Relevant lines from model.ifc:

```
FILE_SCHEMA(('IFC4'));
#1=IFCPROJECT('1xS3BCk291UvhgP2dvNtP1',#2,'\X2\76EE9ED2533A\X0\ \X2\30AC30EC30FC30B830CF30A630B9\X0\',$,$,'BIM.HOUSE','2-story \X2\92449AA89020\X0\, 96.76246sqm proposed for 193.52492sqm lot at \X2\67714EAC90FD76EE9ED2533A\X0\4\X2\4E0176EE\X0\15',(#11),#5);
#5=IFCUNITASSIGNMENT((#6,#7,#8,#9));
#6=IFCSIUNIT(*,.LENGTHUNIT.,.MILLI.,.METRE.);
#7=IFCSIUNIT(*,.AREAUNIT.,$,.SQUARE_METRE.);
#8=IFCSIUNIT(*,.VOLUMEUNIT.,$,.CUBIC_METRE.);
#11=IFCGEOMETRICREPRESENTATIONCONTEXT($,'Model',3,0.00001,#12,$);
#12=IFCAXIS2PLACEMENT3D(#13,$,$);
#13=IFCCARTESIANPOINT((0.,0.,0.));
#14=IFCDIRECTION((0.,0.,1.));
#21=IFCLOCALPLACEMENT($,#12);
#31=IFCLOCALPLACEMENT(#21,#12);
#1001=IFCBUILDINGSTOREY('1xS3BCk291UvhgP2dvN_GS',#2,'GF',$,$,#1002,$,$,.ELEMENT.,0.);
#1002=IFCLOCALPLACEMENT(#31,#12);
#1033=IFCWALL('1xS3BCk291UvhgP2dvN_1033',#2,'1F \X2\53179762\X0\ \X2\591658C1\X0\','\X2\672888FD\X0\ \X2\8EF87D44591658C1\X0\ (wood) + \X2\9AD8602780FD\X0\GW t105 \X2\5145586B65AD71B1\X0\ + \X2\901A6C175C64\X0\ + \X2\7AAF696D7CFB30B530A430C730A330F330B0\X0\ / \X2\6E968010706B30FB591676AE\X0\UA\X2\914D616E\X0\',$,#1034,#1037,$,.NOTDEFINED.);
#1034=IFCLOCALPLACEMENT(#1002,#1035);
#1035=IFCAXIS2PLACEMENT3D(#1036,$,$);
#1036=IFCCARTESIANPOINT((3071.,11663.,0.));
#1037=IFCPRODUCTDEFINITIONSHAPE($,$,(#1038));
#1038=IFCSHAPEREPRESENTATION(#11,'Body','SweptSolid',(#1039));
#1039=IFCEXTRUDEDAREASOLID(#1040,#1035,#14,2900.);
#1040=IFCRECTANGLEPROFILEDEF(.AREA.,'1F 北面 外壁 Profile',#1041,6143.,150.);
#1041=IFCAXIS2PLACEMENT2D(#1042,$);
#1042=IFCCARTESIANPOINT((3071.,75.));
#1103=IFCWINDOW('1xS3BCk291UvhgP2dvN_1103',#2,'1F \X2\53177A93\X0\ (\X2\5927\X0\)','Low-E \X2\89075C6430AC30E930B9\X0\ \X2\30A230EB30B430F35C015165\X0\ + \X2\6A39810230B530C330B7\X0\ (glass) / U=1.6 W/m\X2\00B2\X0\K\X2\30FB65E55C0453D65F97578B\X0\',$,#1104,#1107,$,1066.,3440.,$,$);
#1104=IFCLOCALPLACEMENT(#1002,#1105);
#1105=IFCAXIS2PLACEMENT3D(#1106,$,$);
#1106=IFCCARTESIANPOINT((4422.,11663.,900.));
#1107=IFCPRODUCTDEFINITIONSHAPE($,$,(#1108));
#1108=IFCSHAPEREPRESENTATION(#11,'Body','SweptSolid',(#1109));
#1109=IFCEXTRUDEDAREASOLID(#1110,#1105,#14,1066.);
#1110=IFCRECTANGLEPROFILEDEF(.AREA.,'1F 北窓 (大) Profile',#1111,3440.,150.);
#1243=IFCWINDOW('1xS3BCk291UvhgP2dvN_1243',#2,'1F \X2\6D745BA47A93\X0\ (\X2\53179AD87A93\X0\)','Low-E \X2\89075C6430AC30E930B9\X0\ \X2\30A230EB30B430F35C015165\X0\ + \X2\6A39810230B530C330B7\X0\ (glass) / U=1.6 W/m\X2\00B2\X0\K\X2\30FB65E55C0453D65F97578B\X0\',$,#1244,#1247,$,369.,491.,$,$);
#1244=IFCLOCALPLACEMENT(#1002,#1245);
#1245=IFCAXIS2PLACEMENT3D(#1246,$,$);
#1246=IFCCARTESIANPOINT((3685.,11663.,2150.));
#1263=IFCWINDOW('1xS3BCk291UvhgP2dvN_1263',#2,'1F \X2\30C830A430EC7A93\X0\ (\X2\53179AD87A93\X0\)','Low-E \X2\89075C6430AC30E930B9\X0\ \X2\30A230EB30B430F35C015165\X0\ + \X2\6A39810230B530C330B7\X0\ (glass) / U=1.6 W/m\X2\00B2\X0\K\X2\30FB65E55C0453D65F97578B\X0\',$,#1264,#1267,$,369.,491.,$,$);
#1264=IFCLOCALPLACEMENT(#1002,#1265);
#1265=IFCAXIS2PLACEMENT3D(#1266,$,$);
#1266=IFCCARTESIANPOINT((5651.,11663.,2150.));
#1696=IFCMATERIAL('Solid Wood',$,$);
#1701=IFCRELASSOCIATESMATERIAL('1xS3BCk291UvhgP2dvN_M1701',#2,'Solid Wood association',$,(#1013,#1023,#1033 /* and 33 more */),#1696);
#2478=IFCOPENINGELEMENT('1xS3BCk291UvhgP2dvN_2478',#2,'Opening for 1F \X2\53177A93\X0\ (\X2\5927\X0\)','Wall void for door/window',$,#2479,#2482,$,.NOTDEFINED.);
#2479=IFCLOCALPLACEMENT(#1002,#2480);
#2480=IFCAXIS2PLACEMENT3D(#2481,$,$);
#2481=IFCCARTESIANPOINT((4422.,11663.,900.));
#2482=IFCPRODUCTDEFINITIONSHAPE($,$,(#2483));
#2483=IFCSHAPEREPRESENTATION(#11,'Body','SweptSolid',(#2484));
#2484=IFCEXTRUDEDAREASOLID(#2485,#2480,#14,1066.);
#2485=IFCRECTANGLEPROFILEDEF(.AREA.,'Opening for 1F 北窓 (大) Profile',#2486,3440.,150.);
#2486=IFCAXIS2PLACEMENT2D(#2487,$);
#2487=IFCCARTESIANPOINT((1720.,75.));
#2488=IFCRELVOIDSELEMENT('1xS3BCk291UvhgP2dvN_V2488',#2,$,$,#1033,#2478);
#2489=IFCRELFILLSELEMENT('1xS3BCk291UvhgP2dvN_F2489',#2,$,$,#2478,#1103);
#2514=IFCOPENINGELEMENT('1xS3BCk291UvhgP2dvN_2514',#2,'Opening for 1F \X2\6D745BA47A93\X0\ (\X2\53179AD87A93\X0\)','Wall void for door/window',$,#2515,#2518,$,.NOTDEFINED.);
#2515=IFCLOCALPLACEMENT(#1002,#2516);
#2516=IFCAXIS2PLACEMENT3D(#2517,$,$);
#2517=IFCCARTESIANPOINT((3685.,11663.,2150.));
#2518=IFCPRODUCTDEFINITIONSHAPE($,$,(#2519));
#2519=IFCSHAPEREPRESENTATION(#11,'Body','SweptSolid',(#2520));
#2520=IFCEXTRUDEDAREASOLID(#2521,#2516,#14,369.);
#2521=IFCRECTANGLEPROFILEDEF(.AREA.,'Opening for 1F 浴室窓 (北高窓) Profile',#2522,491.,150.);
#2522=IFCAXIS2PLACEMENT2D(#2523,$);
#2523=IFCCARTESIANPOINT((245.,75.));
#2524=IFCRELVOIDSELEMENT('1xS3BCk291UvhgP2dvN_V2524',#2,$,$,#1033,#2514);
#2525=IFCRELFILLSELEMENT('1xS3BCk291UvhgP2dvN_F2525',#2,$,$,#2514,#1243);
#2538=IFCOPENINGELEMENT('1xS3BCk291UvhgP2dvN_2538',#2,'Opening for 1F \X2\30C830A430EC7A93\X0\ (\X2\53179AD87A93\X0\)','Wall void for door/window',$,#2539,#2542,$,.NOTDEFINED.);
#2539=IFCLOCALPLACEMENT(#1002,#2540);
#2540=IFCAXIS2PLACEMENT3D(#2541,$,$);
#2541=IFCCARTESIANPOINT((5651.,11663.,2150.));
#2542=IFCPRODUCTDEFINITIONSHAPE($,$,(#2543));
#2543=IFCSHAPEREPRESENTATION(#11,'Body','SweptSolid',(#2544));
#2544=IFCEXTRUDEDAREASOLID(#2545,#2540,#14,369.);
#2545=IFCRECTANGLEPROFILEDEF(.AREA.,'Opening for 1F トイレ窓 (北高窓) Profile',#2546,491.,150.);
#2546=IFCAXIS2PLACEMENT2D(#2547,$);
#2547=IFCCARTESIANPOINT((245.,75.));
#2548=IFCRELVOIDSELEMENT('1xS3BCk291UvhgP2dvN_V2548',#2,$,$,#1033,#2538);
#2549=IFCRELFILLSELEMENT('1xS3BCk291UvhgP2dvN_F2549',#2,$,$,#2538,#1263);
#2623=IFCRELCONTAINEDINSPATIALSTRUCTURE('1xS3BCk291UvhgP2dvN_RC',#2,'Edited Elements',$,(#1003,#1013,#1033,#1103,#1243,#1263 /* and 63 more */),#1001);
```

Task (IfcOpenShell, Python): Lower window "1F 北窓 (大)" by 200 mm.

```python
import numpy as np
import ifcopenshell
import ifcopenshell.api.geometry
import ifcopenshell.util.placement
import ifcopenshell.util.unit

model = ifcopenshell.open("model.ifc")
unit_scale = ifcopenshell.util.unit.calculate_unit_scale(model)

window = model.by_guid("1xS3BCk291UvhgP2dvN_1103")
opening = window.FillsVoids[0].RelatingOpeningElement
dz = -200.0

shift = np.array([0.0, 0.0, dz])
# The window is not placed relative to its opening, so move both.
for product in (opening, window):
    matrix = ifcopenshell.util.placement.get_local_placement(product.ObjectPlacement)
    matrix[:3, 3] += shift
    ifcopenshell.api.geometry.edit_object_placement(model, product=product, matrix=matrix, is_si=False)

print(f"moved by {dz * unit_scale:+.3f} m")

model.write("model_edited.ifc")
```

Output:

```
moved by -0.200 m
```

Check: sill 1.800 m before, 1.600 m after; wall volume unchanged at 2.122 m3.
